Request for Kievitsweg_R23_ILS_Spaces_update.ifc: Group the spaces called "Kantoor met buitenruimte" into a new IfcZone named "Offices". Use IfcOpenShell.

First a look at what the model holds.

```python
import ifcopenshell

model = ifcopenshell.open("Kievitsweg_R23_ILS_Spaces_update.ifc")
print(model.schema)
seen = {}
for space in model.by_type("IfcSpace"):
    seen[space.LongName] = seen.get(space.LongName, 0) + 1
for name, count in sorted(seen.items(), key=str):
    print(count, "x", name)
print("zones:", [z.Name for z in model.by_type("IfcZone")][:20])
```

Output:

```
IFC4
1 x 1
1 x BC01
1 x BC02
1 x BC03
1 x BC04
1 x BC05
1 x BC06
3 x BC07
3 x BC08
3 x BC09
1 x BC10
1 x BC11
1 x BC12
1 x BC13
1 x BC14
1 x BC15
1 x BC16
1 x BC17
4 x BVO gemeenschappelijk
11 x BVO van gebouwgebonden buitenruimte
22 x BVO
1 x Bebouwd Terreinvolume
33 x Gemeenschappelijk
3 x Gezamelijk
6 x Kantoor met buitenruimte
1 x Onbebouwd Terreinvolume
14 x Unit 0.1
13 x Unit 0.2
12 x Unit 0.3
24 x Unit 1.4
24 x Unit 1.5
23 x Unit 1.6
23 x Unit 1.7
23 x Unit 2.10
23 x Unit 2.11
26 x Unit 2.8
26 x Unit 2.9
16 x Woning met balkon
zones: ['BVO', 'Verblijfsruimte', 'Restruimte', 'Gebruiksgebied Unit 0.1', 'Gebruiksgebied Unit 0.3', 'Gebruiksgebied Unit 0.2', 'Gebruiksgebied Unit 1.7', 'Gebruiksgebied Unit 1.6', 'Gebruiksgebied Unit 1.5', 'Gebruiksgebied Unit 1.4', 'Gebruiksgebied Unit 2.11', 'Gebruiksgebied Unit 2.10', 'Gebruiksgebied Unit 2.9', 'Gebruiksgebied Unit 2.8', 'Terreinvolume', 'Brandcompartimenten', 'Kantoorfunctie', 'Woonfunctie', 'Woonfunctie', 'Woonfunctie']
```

```python
import ifcopenshell
import ifcopenshell.api.group
import ifcopenshell.api.root

model = ifcopenshell.open("Kievitsweg_R23_ILS_Spaces_update.ifc")

names = {"Kantoor met buitenruimte"}
spaces = [s for s in model.by_type("IfcSpace") if s.LongName in names]

zone = ifcopenshell.api.root.create_entity(model, ifc_class="IfcZone", name="Offices")
ifcopenshell.api.group.assign_group(model, products=spaces, group=zone)
print(len(spaces), "spaces in", zone.Name)

model.write("Kievitsweg_R23_ILS_Spaces_update_v2.ifc")
```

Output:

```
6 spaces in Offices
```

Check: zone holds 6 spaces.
